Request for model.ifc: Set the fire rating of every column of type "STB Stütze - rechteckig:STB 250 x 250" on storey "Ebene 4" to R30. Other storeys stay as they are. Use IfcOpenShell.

First a look at what the model holds.

```python
import ifcopenshell
import ifcopenshell.util.element

model = ifcopenshell.open("model.ifc")
print(model.schema)
storey = next(s for s in model.by_type("IfcBuildingStorey") if s.Name == "Ebene 4")
columns = [e for e in ifcopenshell.util.element.get_decomposition(storey) if e.is_a("IfcColumn")]
seen = {}
for e in columns:
    element_type = ifcopenshell.util.element.get_type(e)
    key = (element_type.Name if element_type != e and element_type else None, ifcopenshell.util.element.get_pset(e, "Pset_ColumnCommon", "FireRating"))
    seen[key] = seen.get(key, 0) + 1
for (name, value), count in sorted(seen.items(), key=str):
    print(count, "x", name, "|", value)
```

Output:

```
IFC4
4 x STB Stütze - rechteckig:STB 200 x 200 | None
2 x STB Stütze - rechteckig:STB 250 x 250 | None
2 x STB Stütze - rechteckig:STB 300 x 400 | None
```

```python
import ifcopenshell
import ifcopenshell.api.pset
import ifcopenshell.util.element

model = ifcopenshell.open("model.ifc")

storey = next(s for s in model.by_type("IfcBuildingStorey") if s.Name == "Ebene 4")
columns = [e for e in ifcopenshell.util.element.get_decomposition(storey) if e.is_a("IfcColumn")]

count = 0
for e in columns:
    element_type = ifcopenshell.util.element.get_type(e)
    if element_type in (None, e) or element_type.Name != "STB Stütze - rechteckig:STB 250 x 250":
        continue
    # add_pset returns the element's existing set when there is one.
    pset = ifcopenshell.api.pset.add_pset(model, product=e, name="Pset_ColumnCommon")
    ifcopenshell.api.pset.edit_pset(model, pset=pset, properties={"FireRating": "R30"})
    count += 1

print(count, "columns updated")

model.write("model_edited.ifc")
```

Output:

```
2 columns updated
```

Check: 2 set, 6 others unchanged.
